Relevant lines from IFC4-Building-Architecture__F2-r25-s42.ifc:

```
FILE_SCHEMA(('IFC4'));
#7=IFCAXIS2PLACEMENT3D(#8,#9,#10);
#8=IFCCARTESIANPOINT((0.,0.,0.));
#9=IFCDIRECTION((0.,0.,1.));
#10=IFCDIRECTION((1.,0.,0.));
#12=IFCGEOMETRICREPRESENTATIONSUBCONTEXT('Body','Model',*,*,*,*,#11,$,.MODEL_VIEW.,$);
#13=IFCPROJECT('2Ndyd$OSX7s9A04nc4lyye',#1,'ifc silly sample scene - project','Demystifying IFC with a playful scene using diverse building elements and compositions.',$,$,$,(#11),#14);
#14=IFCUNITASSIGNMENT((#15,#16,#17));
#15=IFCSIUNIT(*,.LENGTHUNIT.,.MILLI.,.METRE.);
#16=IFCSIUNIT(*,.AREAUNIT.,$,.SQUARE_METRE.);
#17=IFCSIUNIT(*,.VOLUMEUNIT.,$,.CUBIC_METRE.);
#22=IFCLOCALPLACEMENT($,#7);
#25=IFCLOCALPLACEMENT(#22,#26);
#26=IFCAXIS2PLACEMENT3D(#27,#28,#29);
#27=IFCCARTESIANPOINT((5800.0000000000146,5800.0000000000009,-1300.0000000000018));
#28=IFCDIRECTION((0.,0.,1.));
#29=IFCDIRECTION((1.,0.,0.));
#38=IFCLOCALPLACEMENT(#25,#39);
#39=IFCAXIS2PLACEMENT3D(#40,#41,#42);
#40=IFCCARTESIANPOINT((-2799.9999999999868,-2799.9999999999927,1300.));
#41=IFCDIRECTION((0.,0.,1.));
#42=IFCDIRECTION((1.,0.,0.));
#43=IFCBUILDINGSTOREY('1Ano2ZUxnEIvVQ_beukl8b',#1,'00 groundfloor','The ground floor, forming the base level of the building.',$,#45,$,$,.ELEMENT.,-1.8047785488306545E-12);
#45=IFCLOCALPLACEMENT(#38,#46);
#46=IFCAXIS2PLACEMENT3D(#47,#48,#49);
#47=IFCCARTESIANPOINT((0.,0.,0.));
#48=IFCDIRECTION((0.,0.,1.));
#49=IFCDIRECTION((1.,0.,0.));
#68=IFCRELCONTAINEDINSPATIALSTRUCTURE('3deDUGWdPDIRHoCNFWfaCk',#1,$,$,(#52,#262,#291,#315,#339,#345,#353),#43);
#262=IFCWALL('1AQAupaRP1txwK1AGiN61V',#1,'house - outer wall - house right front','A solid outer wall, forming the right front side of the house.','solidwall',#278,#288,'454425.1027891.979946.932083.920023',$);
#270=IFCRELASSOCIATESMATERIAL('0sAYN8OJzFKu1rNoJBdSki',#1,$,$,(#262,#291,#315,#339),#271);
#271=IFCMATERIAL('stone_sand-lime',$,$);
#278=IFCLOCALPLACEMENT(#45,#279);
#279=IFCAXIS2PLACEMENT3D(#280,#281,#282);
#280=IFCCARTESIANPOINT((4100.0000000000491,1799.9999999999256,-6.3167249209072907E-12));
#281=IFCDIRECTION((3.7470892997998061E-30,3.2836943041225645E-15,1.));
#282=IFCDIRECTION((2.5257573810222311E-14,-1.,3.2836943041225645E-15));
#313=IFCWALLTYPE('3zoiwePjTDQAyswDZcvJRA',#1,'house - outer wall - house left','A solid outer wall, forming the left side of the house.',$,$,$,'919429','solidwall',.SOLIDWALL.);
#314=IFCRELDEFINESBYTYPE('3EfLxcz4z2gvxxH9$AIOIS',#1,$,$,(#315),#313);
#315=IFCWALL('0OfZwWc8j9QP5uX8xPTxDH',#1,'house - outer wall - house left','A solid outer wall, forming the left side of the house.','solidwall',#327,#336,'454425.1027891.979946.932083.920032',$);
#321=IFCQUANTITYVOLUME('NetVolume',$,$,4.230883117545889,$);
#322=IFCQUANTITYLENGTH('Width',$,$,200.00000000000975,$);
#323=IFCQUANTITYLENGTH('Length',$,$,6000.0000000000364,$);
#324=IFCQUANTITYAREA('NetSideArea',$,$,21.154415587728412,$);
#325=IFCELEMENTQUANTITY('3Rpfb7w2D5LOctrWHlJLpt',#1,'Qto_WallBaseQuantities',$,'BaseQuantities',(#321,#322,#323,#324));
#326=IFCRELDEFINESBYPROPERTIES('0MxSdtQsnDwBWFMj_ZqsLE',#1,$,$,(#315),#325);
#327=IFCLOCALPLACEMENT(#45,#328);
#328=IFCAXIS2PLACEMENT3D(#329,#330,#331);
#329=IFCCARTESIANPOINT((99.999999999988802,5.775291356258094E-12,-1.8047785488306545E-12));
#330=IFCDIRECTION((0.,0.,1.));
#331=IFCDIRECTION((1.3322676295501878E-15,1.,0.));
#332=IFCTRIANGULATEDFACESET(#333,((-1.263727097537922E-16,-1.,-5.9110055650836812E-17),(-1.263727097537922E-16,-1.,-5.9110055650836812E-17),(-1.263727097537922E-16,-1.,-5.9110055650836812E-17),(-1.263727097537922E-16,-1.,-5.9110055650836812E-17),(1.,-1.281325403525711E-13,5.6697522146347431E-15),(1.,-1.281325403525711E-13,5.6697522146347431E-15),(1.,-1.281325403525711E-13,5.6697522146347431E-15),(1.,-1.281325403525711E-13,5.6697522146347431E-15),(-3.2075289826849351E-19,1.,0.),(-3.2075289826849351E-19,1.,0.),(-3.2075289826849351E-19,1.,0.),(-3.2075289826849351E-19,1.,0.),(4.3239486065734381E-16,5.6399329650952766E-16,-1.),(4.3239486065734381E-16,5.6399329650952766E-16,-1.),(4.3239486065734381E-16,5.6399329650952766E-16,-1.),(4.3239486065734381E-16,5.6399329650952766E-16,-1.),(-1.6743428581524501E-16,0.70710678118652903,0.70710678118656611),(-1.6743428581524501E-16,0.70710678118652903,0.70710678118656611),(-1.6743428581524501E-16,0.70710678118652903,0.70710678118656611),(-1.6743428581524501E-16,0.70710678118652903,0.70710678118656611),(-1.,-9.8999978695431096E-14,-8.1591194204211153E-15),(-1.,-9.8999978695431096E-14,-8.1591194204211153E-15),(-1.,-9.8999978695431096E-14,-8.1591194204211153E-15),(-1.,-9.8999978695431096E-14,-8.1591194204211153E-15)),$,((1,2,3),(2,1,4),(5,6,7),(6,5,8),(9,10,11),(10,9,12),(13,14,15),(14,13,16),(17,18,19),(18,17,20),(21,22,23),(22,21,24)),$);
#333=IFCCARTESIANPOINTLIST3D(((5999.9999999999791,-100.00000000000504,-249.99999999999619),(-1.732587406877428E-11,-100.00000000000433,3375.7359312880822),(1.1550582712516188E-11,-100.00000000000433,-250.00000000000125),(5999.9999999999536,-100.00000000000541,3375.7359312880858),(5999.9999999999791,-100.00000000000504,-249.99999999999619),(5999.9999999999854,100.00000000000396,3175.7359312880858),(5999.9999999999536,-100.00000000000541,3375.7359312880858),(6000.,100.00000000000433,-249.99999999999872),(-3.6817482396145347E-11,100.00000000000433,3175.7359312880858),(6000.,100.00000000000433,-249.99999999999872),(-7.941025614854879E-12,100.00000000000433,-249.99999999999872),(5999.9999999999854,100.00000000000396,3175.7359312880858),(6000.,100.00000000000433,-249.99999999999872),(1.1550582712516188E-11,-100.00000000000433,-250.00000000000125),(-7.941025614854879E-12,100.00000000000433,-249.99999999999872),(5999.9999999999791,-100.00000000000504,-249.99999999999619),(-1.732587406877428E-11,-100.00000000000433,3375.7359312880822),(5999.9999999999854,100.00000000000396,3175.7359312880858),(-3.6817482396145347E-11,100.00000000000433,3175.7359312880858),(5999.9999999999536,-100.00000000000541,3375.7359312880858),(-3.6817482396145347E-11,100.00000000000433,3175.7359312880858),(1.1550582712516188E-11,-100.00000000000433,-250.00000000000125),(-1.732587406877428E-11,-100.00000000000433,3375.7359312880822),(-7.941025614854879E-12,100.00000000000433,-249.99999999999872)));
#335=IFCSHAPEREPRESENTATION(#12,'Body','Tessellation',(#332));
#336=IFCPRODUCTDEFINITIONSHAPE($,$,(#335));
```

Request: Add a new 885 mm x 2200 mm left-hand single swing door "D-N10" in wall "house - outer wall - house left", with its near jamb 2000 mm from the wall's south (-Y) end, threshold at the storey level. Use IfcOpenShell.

```python
import numpy as np
import ifcopenshell
import ifcopenshell.api.feature
import ifcopenshell.api.geometry
import ifcopenshell.api.pset
import ifcopenshell.api.root
import ifcopenshell.api.spatial
import ifcopenshell.geom
import ifcopenshell.util.element
import ifcopenshell.util.placement
import ifcopenshell.util.representation
import ifcopenshell.util.shape
import ifcopenshell.util.unit

model = ifcopenshell.open("IFC4-Building-Architecture__F2-r25-s42.ifc")
unit_scale = ifcopenshell.util.unit.calculate_unit_scale(model)
area_scale = ifcopenshell.util.unit.calculate_unit_scale(model, "AREAUNIT")
volume_scale = ifcopenshell.util.unit.calculate_unit_scale(model, "VOLUMEUNIT")
settings = ifcopenshell.geom.settings()


def volume(element):
    """Net volume in cubic metres, openings subtracted."""
    shape = ifcopenshell.geom.create_shape(settings, element)
    return ifcopenshell.util.shape.get_volume(shape.geometry)


wall = model.by_id(315)
storey = ifcopenshell.util.element.get_container(wall, ifc_class="IfcBuildingStorey")
context = ifcopenshell.util.representation.get_context(model, "Model", "Body", "MODEL_VIEW")
before = volume(wall)

width, height, from_end, sill = 0.885, 2.2, 2, 0.0  # metres

# The wall runs along its own X axis, and the end named is its -X end.
wall_shape = ifcopenshell.geom.create_shape(settings, wall)
x, y, z = ifcopenshell.util.shape.get_vertices(wall_shape.geometry).T
start = x.min() + from_end
face, thickness = float(y.min()), float(y.max() - y.min())
wall_matrix = ifcopenshell.util.placement.get_local_placement(wall.ObjectPlacement)
level = ifcopenshell.util.placement.get_local_placement(storey.ObjectPlacement)[2, 3]


def in_wall(x, y):
    """Placement at x, y metres in the wall's axes, at sill height."""
    matrix = wall_matrix.copy()
    matrix[:, 3] = wall_matrix @ np.array([x / unit_scale, y / unit_scale, 0.0, 1.0])
    matrix[2, 3] = level + sill / unit_scale
    return matrix


# Opening: a box that overshoots both wall faces by 50 mm.
opening = ifcopenshell.api.root.create_entity(model, ifc_class="IfcOpeningElement", predefined_type="OPENING")
box = ifcopenshell.api.geometry.add_wall_representation(
    model, context=context, length=width, height=height, thickness=thickness + 0.1
)
ifcopenshell.api.geometry.assign_representation(model, product=opening, representation=box)
ifcopenshell.api.geometry.edit_object_placement(model, product=opening, matrix=in_wall(start, face - 0.05), is_si=False)
ifcopenshell.api.feature.add_feature(model, feature=opening, element=wall)

door = ifcopenshell.api.root.create_entity(model, ifc_class="IfcDoor", name="D-N10", predefined_type="DOOR")
door.OverallWidth, door.OverallHeight = width / unit_scale, height / unit_scale
door.OperationType = "SINGLE_SWING_LEFT"
body = ifcopenshell.api.geometry.add_door_representation(
    model,
    context=context,
    overall_width=door.OverallWidth,
    overall_height=door.OverallHeight,
    operation_type="SINGLE_SWING_LEFT",
    lining_properties={"LiningDepth": thickness / unit_scale, "ThresholdDepth": thickness / unit_scale},
)
ifcopenshell.api.geometry.assign_representation(model, product=door, representation=body)
ifcopenshell.api.spatial.assign_container(model, products=[door], relating_structure=storey)
ifcopenshell.api.feature.add_filling(model, opening=opening, element=door)

# The lining spans the wall, so the door starts at the wall face.
ifcopenshell.api.geometry.edit_object_placement(model, product=door, matrix=in_wall(start, face), is_si=False)

after = volume(wall)

# Update the wall's stored quantities.
qto = model.by_id(ifcopenshell.util.element.get_pset(wall, "Qto_WallBaseQuantities", should_inherit=False)["id"])
ifcopenshell.api.pset.edit_qto(model, qto=qto, properties={
    "NetVolume": after / volume_scale,
    "NetSideArea": after / thickness / area_scale,
})

print(f"wall volume {before:.3f} -> {after:.3f} m3")

model.write("IFC4-Building-Architecture__F2-r25-s42_updated.ifc")
```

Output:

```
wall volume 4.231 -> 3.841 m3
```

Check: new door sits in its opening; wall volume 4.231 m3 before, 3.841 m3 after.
